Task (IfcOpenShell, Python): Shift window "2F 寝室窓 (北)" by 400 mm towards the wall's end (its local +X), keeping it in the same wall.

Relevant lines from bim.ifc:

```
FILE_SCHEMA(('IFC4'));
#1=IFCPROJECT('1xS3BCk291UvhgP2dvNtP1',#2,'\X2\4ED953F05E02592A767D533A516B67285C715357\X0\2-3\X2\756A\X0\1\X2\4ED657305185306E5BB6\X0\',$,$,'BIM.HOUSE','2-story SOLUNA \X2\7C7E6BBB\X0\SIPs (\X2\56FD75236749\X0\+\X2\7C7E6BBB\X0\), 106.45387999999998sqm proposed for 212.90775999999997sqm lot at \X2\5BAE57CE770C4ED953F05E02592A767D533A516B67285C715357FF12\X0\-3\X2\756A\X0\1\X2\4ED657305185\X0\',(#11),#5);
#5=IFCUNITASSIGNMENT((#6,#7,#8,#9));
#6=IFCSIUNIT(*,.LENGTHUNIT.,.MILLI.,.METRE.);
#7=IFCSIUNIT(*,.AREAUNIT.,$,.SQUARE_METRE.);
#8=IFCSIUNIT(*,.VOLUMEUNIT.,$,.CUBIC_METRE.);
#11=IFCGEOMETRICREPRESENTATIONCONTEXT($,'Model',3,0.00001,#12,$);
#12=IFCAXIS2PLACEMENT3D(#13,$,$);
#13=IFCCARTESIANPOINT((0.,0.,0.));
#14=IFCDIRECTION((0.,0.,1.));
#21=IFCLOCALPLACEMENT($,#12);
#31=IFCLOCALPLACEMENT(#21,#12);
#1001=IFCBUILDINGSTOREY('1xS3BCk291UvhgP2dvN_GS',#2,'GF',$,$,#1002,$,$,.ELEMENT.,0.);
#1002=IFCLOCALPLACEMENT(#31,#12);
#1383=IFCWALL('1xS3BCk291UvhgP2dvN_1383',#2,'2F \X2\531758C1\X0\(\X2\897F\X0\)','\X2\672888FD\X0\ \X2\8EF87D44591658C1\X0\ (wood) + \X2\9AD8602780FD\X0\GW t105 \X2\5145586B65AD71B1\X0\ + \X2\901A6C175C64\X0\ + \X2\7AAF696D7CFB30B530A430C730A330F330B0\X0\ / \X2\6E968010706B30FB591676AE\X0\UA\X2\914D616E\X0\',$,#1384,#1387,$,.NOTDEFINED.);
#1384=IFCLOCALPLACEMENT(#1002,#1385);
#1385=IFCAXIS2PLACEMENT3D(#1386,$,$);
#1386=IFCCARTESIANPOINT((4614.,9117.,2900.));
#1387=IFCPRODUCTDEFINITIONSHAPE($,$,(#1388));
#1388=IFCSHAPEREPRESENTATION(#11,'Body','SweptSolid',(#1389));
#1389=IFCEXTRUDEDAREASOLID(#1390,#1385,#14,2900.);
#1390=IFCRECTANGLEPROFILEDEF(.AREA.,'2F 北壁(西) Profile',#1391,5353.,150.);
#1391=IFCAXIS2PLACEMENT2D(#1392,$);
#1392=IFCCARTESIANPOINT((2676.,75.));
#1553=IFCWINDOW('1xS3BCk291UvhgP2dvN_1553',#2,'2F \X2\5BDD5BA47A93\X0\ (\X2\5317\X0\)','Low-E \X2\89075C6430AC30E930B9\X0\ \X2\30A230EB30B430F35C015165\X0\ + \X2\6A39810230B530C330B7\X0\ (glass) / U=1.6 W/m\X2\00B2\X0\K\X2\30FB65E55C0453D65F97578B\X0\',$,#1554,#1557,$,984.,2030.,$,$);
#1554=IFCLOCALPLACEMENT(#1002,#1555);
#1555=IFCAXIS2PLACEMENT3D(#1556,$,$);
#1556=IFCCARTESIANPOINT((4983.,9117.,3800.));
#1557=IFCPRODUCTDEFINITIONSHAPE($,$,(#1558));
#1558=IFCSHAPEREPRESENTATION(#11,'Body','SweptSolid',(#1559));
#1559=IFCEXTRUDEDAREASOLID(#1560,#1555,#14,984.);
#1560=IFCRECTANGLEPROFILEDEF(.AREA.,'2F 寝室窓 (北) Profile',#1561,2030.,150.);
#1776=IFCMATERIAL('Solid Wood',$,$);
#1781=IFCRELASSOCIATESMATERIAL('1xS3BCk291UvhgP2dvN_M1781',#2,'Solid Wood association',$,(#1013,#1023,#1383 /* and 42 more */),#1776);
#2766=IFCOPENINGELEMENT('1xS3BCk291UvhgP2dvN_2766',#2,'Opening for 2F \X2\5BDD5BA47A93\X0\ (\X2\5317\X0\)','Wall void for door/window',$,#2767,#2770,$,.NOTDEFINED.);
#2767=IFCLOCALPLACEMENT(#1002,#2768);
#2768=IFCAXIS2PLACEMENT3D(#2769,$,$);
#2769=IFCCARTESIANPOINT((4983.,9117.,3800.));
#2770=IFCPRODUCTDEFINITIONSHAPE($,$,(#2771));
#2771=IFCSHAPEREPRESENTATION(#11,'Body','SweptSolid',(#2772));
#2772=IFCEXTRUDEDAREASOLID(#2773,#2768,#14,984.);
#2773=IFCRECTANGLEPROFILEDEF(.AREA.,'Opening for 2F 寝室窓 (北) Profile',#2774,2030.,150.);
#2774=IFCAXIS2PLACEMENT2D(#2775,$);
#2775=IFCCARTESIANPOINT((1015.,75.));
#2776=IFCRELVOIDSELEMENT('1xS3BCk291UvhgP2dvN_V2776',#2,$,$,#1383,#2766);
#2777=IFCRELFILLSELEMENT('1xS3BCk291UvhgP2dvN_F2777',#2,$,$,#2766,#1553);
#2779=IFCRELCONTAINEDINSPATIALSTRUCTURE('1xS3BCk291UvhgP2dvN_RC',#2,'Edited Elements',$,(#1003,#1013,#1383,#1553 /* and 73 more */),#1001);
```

```python
import ifcopenshell
import ifcopenshell.api.geometry
import ifcopenshell.util.placement

model = ifcopenshell.open("bim.ifc")

window = model.by_guid("1xS3BCk291UvhgP2dvN_1553")
opening = window.FillsVoids[0].RelatingOpeningElement
wall = opening.VoidsElements[0].RelatingBuildingElement

wall_matrix = ifcopenshell.util.placement.get_local_placement(wall.ObjectPlacement)
shift = wall_matrix[:3, 0] * 400.0
before = ifcopenshell.util.placement.get_local_placement(window.ObjectPlacement)[:3, 3].copy()

# The window is not placed relative to its opening, so move both.
for product in (opening, window):
    matrix = ifcopenshell.util.placement.get_local_placement(product.ObjectPlacement)
    matrix[:3, 3] += shift
    ifcopenshell.api.geometry.edit_object_placement(model, product=product, matrix=matrix, is_si=False)

after = ifcopenshell.util.placement.get_local_placement(window.ObjectPlacement)[:3, 3]
print("window moved by", (after - before).round(3) + 0.0)

model.write("bim_rev.ifc")
```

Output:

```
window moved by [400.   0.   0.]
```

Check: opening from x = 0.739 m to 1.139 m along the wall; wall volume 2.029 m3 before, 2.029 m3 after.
